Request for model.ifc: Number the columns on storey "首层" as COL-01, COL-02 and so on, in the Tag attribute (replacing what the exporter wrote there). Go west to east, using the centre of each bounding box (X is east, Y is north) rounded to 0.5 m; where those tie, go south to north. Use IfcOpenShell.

First a look at what the model holds.

```python
import ifcopenshell
import ifcopenshell.util.element
import ifcopenshell.util.placement

model = ifcopenshell.open("model.ifc")
print(model.schema)
storey = next(s for s in model.by_type("IfcBuildingStorey") if s.Name == "首层")
columns = [e for e in ifcopenshell.util.element.get_decomposition(storey) if e.is_a("IfcColumn")]
for e in sorted(columns, key=lambda e: e.id()):
    origin = ifcopenshell.util.placement.get_local_placement(e.ObjectPlacement)[:3, 3]
    print(e.id(), e.Tag, e.Name, origin.round(2) + 0.0, sep=" | ")
```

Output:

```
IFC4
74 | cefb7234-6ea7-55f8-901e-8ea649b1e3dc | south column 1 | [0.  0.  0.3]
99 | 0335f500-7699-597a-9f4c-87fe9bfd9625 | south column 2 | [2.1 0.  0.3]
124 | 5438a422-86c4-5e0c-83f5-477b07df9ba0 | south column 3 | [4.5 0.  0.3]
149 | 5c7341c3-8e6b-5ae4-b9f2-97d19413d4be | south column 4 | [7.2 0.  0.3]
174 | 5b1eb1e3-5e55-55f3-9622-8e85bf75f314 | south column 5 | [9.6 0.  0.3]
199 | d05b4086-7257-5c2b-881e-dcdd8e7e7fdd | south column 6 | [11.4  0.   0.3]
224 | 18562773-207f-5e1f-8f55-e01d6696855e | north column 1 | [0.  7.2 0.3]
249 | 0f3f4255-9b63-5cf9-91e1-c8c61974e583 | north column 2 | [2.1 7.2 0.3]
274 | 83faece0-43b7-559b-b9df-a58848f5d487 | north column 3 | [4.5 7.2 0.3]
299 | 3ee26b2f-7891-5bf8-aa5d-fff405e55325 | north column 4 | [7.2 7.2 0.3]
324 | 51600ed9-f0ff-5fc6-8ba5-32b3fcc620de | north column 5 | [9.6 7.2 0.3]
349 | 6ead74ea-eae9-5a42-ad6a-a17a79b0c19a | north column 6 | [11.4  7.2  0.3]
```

```python
import ifcopenshell
import ifcopenshell.geom
import ifcopenshell.util.element
import ifcopenshell.util.shape

model = ifcopenshell.open("model.ifc")
settings = ifcopenshell.geom.settings()
settings.set("use-world-coords", True)


def centre(element):
    shape = ifcopenshell.geom.create_shape(settings, element)
    return ifcopenshell.util.shape.get_bbox_centroid(shape.geometry)


storey = next(s for s in model.by_type("IfcBuildingStorey") if s.Name == "首层")
columns = [e for e in ifcopenshell.util.element.get_decomposition(storey) if e.is_a("IfcColumn")]

# Insertion points can sit at a corner or the storey origin, so sort by the geometry (in metres).
centres = {e: centre(e) for e in columns}
columns.sort(key=lambda e: (round(centres[e][0] / 0.5), centres[e][1]))

for i, e in enumerate(columns, start=1):
    number = f"COL-{i:02d}"
    e.Tag = number
    print(e.id(), number)

model.write("model_v2.ifc")
```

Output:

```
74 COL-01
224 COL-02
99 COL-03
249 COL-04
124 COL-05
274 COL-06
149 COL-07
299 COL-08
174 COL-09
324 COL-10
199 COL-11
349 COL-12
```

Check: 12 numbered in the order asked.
